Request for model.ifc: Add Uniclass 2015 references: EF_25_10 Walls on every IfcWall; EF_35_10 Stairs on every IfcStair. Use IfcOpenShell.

First a look at what the model holds.

```python
import ifcopenshell

model = ifcopenshell.open("model.ifc")
print(model.schema)
print("classifications:", [c.Name for c in model.by_type("IfcClassification")])
for ifc_class in ("IfcDoor", "IfcRoof", "IfcStair", "IfcWall", "IfcWindow"):
    print(ifc_class, len(model.by_type(ifc_class)))
```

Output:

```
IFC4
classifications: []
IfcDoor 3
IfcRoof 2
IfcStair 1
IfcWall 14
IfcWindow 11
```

```python
import ifcopenshell
import ifcopenshell.api.classification

model = ifcopenshell.open("model.ifc")

system = ifcopenshell.api.classification.add_classification(model, classification="Uniclass 2015")

codes = {
    "IfcWall": ("EF_25_10", "Walls"),
    "IfcStair": ("EF_35_10", "Stairs"),
}
for ifc_class, (code, name) in codes.items():
    products = model.by_type(ifc_class)
    ifcopenshell.api.classification.add_reference(
        model, products=products, classification=system, identification=code, name=name
    )
    print(code, len(products))

model.write("model_v2.ifc")
```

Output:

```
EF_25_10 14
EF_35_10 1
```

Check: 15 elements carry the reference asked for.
